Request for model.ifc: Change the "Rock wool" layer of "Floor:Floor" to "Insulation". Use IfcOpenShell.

First a look at what the model holds.

```python
import ifcopenshell
import ifcopenshell.util.element

model = ifcopenshell.open("model.ifc")
print(model.schema)
for layer_set in model.by_type("IfcMaterialLayerSet"):
    if layer_set.LayerSetName == "Floor:Floor":
        for layer in layer_set.MaterialLayers:
            print(layer.id(), layer.Material and layer.Material.Name, layer.LayerThickness, sep=" | ")
        print(len(ifcopenshell.util.element.get_elements_by_material(model, layer_set)), "elements and types use it")
print(sorted(m.Name for m in model.by_type("IfcMaterial") if m.Name)[:60])
```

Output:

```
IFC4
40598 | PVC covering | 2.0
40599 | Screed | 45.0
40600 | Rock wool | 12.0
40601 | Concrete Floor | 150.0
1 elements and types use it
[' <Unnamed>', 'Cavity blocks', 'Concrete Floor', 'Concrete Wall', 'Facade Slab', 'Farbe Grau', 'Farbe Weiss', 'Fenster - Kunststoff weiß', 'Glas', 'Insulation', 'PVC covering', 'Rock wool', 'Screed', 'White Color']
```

```python
import ifcopenshell
import ifcopenshell.api.material

model = ifcopenshell.open("model.ifc")

layer_set = next(s for s in model.by_type("IfcMaterialLayerSet") if s.LayerSetName == "Floor:Floor")
layer = next(l for l in layer_set.MaterialLayers if l.Material and l.Material.Name == "Rock wool")
material = next(m for m in model.by_type("IfcMaterial") if m.Name == "Insulation")

# Point this one layer at the other material; renaming the old one would change it everywhere.
ifcopenshell.api.material.edit_layer(model, layer=layer, attributes={}, material=material)

print([l.Material.Name if l.Material else None for l in layer_set.MaterialLayers])

model.write("model_rev.ifc")
```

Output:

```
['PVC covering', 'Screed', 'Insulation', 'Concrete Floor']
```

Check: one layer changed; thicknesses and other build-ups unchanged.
